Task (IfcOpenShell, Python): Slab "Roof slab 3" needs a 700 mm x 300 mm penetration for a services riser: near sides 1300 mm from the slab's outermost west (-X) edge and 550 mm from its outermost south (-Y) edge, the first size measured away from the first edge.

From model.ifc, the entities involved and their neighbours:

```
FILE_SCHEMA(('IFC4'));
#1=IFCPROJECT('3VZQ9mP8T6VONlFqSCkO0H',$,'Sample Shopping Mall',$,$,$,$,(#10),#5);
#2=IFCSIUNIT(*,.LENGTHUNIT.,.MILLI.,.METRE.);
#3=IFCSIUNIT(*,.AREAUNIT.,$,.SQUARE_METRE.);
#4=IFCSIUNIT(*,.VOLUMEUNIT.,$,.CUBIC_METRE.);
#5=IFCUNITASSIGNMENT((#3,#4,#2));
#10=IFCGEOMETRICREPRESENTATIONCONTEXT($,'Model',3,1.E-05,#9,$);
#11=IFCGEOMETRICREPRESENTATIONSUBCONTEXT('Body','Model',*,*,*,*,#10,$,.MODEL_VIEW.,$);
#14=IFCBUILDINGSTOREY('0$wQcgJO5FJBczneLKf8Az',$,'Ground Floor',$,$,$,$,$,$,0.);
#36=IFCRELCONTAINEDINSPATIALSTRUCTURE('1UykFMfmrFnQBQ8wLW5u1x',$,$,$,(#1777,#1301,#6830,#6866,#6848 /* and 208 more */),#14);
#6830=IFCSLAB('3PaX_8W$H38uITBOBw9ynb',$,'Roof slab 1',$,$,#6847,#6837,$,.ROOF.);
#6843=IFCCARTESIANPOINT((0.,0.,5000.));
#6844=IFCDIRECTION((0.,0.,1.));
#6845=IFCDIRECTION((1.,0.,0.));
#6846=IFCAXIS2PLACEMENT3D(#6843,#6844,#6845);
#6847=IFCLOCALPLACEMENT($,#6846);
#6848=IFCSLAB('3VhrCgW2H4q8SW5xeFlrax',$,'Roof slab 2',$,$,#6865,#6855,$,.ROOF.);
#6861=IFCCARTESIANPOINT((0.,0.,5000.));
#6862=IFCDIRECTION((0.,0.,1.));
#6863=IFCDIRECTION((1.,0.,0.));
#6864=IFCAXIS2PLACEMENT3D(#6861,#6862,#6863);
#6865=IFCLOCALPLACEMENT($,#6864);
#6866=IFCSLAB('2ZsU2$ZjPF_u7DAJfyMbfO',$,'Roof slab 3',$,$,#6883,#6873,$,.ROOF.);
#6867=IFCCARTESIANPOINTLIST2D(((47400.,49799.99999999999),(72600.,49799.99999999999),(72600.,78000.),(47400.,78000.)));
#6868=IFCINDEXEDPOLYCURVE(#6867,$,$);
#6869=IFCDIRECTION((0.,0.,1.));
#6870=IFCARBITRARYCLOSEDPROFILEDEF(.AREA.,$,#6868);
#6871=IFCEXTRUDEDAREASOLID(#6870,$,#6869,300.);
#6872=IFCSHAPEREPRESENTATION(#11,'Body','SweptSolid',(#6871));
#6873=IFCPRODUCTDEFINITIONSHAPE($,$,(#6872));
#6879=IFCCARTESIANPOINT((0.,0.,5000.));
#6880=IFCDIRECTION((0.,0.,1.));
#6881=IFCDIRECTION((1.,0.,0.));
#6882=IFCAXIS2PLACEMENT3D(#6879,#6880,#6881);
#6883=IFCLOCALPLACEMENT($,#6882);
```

```python
import numpy as np
import ifcopenshell
import ifcopenshell.api.feature
import ifcopenshell.api.geometry
import ifcopenshell.api.root
import ifcopenshell.geom
import ifcopenshell.util.placement
import ifcopenshell.util.representation
import ifcopenshell.util.shape
import ifcopenshell.util.unit

model = ifcopenshell.open("model.ifc")
unit_scale = ifcopenshell.util.unit.calculate_unit_scale(model)
settings = ifcopenshell.geom.settings()


def volume(element):
    """Net volume in cubic metres, openings subtracted."""
    shape = ifcopenshell.geom.create_shape(settings, element)
    return ifcopenshell.util.shape.get_volume(shape.geometry)


slab = model.by_guid("2ZsU2$ZjPF_u7DAJfyMbfO")
before = volume(slab)

# Extent in the slab's own axes, in metres. The edges named are its -X and -Y sides.
slab_shape = ifcopenshell.geom.create_shape(settings, slab)
vertices = ifcopenshell.util.shape.get_vertices(slab_shape.geometry)
x_min, y_min, bottom = vertices.min(axis=0)
top = vertices[:, 2].max()

opening = ifcopenshell.api.root.create_entity(model, ifc_class="IfcOpeningElement", name="Services riser opening", predefined_type="OPENING")
context = ifcopenshell.util.representation.get_context(model, "Model", "Body", "MODEL_VIEW")
width, depth = 0.7, 0.3
outline = [(0.0, 0.0), (width, 0.0), (width, depth), (0.0, depth), (0.0, 0.0)]
# Overshoot both faces by 50 mm so the cut is clean.
shape = ifcopenshell.api.geometry.add_slab_representation(
    model, context=context, depth=top - bottom + 0.1, polyline=outline
)
ifcopenshell.api.geometry.assign_representation(model, product=opening, representation=shape)

matrix = ifcopenshell.util.placement.get_local_placement(slab.ObjectPlacement)
matrix[:, 3] = matrix @ np.append(np.array([x_min + 1.3, y_min + 0.55, bottom - 0.05]) / unit_scale, 1.0)
ifcopenshell.api.geometry.edit_object_placement(model, product=opening, matrix=matrix, is_si=False)
ifcopenshell.api.feature.add_feature(model, feature=opening, element=slab)

after = volume(slab)

print(f"slab volume {before:.3f} -> {after:.3f} m3")

model.write("model_updated.ifc")
```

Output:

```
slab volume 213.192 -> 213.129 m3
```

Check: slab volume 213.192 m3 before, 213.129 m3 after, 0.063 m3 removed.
